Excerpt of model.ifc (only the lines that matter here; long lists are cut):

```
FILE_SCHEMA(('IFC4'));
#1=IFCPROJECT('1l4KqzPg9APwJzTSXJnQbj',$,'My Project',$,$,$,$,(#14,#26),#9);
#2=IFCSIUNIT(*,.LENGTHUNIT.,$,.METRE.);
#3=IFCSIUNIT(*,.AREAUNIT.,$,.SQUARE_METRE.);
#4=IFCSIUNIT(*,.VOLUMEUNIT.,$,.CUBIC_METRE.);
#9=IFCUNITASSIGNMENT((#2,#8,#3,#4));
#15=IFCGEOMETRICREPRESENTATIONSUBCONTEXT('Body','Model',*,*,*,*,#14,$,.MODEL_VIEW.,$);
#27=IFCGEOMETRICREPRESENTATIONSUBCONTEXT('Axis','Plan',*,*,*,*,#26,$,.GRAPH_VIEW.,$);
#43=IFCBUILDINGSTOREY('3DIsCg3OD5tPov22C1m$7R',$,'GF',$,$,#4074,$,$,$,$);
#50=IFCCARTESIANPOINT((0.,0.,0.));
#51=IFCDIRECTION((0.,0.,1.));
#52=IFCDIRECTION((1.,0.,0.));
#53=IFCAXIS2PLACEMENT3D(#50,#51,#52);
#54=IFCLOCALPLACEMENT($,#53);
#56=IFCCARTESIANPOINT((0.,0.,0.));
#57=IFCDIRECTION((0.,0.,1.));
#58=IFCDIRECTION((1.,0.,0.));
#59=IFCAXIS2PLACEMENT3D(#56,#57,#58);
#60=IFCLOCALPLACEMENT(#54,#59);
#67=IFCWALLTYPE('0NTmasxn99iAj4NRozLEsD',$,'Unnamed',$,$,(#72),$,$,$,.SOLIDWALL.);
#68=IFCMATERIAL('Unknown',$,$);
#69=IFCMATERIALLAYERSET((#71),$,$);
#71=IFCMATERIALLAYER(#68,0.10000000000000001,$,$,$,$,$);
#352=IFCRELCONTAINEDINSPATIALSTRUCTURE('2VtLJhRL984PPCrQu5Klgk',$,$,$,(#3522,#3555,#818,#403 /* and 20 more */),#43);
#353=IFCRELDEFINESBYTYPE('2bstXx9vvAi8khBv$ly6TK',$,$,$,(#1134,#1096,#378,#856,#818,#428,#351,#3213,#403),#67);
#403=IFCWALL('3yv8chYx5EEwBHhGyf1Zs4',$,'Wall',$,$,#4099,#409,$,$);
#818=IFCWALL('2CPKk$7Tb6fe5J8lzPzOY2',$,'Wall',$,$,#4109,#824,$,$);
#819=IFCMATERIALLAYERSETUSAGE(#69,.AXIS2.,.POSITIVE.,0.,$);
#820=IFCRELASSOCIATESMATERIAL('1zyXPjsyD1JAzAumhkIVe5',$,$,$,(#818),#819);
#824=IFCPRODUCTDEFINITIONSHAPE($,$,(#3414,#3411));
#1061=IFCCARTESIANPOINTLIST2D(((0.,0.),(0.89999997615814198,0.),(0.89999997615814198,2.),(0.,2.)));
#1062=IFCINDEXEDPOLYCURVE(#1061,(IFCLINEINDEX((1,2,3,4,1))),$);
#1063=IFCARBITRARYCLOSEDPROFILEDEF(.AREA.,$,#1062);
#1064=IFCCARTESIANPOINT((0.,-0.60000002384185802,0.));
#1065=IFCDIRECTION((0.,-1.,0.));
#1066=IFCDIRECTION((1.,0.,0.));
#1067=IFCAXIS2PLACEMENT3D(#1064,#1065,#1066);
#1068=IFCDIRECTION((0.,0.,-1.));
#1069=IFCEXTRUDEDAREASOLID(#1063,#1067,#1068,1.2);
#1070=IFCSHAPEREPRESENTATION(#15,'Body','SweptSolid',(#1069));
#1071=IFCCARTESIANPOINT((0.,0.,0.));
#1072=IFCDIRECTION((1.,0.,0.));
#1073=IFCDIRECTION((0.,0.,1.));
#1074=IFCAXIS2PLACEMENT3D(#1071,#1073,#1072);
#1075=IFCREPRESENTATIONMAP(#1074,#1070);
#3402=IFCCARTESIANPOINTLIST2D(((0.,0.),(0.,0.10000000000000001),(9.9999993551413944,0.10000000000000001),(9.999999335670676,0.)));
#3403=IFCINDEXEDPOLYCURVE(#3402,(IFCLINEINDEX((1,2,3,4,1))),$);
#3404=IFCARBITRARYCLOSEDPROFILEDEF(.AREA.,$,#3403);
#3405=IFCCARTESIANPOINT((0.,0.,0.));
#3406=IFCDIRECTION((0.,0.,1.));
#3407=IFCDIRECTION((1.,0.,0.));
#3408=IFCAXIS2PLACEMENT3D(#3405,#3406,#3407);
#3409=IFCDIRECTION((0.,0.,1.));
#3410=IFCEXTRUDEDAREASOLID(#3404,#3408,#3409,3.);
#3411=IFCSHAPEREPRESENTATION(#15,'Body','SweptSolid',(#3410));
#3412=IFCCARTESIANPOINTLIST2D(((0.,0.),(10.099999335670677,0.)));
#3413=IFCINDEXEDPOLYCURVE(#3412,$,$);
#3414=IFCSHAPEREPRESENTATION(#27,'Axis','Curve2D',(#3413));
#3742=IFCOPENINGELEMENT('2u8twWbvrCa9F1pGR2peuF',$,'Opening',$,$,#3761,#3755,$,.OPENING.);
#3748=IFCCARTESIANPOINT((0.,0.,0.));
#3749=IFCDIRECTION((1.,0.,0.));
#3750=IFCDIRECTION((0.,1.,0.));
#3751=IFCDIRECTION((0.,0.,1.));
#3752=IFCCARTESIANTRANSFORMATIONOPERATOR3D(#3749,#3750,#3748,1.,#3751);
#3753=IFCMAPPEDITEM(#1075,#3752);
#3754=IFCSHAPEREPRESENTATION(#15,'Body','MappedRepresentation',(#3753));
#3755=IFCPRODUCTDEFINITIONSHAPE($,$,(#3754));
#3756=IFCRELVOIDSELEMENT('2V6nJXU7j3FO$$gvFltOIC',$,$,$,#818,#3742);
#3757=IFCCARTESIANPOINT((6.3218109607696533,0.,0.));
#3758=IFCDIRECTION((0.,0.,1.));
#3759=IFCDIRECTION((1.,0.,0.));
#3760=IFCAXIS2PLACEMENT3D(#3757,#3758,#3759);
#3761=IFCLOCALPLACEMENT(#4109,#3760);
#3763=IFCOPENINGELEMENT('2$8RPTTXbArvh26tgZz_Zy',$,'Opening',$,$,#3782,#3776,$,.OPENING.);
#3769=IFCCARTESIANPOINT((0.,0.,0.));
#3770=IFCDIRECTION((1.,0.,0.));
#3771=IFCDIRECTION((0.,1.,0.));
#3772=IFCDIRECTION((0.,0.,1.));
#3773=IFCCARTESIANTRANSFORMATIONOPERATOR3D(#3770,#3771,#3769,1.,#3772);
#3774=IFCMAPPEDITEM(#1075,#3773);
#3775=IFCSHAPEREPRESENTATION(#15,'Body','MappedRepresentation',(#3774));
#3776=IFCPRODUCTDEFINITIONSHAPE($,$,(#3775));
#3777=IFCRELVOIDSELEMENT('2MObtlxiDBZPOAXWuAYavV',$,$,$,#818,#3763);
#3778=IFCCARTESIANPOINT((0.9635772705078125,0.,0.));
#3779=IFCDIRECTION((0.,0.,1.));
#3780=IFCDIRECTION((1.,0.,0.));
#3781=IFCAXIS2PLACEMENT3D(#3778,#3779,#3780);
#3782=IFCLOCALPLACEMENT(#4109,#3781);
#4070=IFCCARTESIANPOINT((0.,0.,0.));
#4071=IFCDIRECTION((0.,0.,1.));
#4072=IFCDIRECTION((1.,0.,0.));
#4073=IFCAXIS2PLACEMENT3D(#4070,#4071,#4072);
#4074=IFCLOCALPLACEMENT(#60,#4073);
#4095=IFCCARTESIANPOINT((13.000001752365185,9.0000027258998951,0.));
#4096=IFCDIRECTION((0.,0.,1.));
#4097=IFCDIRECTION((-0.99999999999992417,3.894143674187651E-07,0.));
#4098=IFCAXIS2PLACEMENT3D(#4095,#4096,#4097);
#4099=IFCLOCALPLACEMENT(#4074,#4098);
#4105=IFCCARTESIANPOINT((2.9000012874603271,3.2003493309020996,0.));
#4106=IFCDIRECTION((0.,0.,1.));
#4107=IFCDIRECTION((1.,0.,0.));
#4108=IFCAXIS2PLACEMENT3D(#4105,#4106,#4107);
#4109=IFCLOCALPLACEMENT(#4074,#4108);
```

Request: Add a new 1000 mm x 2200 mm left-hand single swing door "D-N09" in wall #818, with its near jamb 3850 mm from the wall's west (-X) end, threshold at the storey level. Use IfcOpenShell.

```python
import numpy as np
import ifcopenshell
import ifcopenshell.api.feature
import ifcopenshell.api.geometry
import ifcopenshell.api.root
import ifcopenshell.api.spatial
import ifcopenshell.geom
import ifcopenshell.util.element
import ifcopenshell.util.placement
import ifcopenshell.util.representation
import ifcopenshell.util.shape
import ifcopenshell.util.unit

model = ifcopenshell.open("model.ifc")
unit_scale = ifcopenshell.util.unit.calculate_unit_scale(model)
settings = ifcopenshell.geom.settings()


def volume(element):
    """Net volume in cubic metres, openings subtracted."""
    shape = ifcopenshell.geom.create_shape(settings, element)
    return ifcopenshell.util.shape.get_volume(shape.geometry)


wall = model.by_id(818)
storey = ifcopenshell.util.element.get_container(wall, ifc_class="IfcBuildingStorey")
context = ifcopenshell.util.representation.get_context(model, "Model", "Body", "MODEL_VIEW")
before = volume(wall)

width, height, from_end, sill = 1, 2.2, 3.85, 0.0  # metres

# The wall runs along its own X axis, and the end named is its -X end.
wall_shape = ifcopenshell.geom.create_shape(settings, wall)
x, y, z = ifcopenshell.util.shape.get_vertices(wall_shape.geometry).T
start = x.min() + from_end
face, thickness = float(y.min()), float(y.max() - y.min())
wall_matrix = ifcopenshell.util.placement.get_local_placement(wall.ObjectPlacement)
level = ifcopenshell.util.placement.get_local_placement(storey.ObjectPlacement)[2, 3]


def in_wall(x, y):
    """Placement at x, y metres in the wall's axes, at sill height."""
    matrix = wall_matrix.copy()
    matrix[:, 3] = wall_matrix @ np.array([x / unit_scale, y / unit_scale, 0.0, 1.0])
    matrix[2, 3] = level + sill / unit_scale
    return matrix


# Opening: a box that overshoots both wall faces by 50 mm.
opening = ifcopenshell.api.root.create_entity(model, ifc_class="IfcOpeningElement", predefined_type="OPENING")
box = ifcopenshell.api.geometry.add_wall_representation(
    model, context=context, length=width, height=height, thickness=thickness + 0.1
)
ifcopenshell.api.geometry.assign_representation(model, product=opening, representation=box)
ifcopenshell.api.geometry.edit_object_placement(model, product=opening, matrix=in_wall(start, face - 0.05), is_si=False)
ifcopenshell.api.feature.add_feature(model, feature=opening, element=wall)

door = ifcopenshell.api.root.create_entity(model, ifc_class="IfcDoor", name="D-N09", predefined_type="DOOR")
door.OverallWidth, door.OverallHeight = width / unit_scale, height / unit_scale
door.OperationType = "SINGLE_SWING_LEFT"
body = ifcopenshell.api.geometry.add_door_representation(
    model,
    context=context,
    overall_width=door.OverallWidth,
    overall_height=door.OverallHeight,
    operation_type="SINGLE_SWING_LEFT",
    lining_properties={"LiningDepth": thickness / unit_scale, "ThresholdDepth": thickness / unit_scale},
)
ifcopenshell.api.geometry.assign_representation(model, product=door, representation=body)
ifcopenshell.api.spatial.assign_container(model, products=[door], relating_structure=storey)
ifcopenshell.api.feature.add_filling(model, opening=opening, element=door)

# The lining spans the wall, so the door starts at the wall face.
ifcopenshell.api.geometry.edit_object_placement(model, product=door, matrix=in_wall(start, face), is_si=False)

after = volume(wall)

print(f"wall volume {before:.3f} -> {after:.3f} m3")

model.write("model_v2.ifc")
```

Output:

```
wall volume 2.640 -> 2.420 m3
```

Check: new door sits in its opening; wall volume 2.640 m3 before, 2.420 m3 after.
